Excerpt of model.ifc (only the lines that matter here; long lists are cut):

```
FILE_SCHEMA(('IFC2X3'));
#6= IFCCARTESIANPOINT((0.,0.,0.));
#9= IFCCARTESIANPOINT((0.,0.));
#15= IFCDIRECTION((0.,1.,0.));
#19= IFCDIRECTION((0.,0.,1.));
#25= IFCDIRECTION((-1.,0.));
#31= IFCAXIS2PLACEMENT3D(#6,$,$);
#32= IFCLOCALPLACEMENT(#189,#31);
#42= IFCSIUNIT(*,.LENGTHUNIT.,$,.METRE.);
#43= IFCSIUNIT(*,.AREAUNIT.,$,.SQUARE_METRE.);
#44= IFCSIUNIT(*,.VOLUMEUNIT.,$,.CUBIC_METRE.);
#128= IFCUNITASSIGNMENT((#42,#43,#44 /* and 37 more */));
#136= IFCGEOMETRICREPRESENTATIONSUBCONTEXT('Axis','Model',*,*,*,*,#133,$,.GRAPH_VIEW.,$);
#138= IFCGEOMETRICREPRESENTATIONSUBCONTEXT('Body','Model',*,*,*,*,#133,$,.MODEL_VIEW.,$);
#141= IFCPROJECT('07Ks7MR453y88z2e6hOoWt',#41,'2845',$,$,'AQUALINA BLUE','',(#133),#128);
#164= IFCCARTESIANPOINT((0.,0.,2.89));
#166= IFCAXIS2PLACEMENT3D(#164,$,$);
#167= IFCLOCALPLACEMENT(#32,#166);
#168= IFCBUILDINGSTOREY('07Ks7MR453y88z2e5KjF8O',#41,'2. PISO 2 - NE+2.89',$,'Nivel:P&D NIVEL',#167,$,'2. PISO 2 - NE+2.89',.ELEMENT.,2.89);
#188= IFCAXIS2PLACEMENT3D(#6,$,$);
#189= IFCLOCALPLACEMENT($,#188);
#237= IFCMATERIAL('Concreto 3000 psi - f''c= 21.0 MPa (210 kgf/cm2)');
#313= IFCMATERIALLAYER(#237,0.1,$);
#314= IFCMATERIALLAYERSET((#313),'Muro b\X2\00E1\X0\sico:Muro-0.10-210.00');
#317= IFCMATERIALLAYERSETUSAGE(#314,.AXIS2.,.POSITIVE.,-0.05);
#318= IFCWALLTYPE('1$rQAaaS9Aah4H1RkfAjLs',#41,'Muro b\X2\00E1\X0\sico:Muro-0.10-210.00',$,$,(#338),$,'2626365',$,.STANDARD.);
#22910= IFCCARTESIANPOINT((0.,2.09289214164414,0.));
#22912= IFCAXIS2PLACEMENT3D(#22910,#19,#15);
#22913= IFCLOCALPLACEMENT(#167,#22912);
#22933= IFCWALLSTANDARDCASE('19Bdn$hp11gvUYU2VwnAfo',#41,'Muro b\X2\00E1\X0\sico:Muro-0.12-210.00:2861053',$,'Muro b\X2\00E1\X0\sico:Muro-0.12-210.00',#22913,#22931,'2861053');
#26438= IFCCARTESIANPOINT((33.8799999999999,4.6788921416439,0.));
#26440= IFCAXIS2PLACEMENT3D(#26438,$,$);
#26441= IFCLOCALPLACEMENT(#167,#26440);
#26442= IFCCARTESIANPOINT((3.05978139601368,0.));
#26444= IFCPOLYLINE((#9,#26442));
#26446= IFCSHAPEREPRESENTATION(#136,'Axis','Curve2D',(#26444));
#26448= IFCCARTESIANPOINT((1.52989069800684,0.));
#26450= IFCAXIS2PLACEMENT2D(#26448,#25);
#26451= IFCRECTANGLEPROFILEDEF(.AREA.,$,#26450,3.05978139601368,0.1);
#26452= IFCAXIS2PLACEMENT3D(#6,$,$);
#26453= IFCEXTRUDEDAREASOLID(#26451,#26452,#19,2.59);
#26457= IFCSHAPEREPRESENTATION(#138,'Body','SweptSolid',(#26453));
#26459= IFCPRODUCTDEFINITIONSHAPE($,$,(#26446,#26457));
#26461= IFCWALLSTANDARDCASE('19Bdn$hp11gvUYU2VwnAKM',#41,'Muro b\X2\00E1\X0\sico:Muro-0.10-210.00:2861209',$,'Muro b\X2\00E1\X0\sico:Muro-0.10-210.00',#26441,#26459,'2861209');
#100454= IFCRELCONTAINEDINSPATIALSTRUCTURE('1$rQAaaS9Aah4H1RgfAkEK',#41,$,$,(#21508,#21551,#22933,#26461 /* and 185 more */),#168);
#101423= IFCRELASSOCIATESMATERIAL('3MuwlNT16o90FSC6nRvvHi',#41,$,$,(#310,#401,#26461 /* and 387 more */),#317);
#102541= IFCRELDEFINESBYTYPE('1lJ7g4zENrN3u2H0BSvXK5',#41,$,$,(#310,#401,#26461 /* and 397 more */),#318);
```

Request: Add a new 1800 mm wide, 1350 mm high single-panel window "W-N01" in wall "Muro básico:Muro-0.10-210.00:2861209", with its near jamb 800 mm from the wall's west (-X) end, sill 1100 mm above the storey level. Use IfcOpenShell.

```python
import numpy as np
import ifcopenshell
import ifcopenshell.api.feature
import ifcopenshell.api.geometry
import ifcopenshell.api.root
import ifcopenshell.api.spatial
import ifcopenshell.api.type
import ifcopenshell.geom
import ifcopenshell.util.element
import ifcopenshell.util.placement
import ifcopenshell.util.representation
import ifcopenshell.util.shape
import ifcopenshell.util.unit

model = ifcopenshell.open("model.ifc")
unit_scale = ifcopenshell.util.unit.calculate_unit_scale(model)
settings = ifcopenshell.geom.settings()


def volume(element):
    """Net volume in cubic metres, openings subtracted."""
    shape = ifcopenshell.geom.create_shape(settings, element)
    return ifcopenshell.util.shape.get_volume(shape.geometry)


wall = model.by_guid("19Bdn$hp11gvUYU2VwnAKM")
storey = ifcopenshell.util.element.get_container(wall, ifc_class="IfcBuildingStorey")
context = ifcopenshell.util.representation.get_context(model, "Model", "Body", "MODEL_VIEW")
before = volume(wall)

width, height, from_end, sill = 1.8, 1.35, 0.8, 1.1  # metres

# The wall runs along its own X axis, and the end named is its -X end.
wall_shape = ifcopenshell.geom.create_shape(settings, wall)
x, y, z = ifcopenshell.util.shape.get_vertices(wall_shape.geometry).T
start = x.min() + from_end
face, thickness = float(y.min()), float(y.max() - y.min())
wall_matrix = ifcopenshell.util.placement.get_local_placement(wall.ObjectPlacement)
level = ifcopenshell.util.placement.get_local_placement(storey.ObjectPlacement)[2, 3]


def in_wall(x, y):
    """Placement at x, y metres in the wall's axes, at sill height."""
    matrix = wall_matrix.copy()
    matrix[:, 3] = wall_matrix @ np.array([x / unit_scale, y / unit_scale, 0.0, 1.0])
    matrix[2, 3] = level + sill / unit_scale
    return matrix


# Opening: a box that overshoots both wall faces by 50 mm.
opening = ifcopenshell.api.root.create_entity(model, ifc_class="IfcOpeningElement")
box = ifcopenshell.api.geometry.add_wall_representation(
    model, context=context, length=width, height=height, thickness=thickness + 0.1
)
ifcopenshell.api.geometry.assign_representation(model, product=opening, representation=box)
ifcopenshell.api.geometry.edit_object_placement(model, product=opening, matrix=in_wall(start, face - 0.05), is_si=False)
ifcopenshell.api.feature.add_feature(model, feature=opening, element=wall)

window = ifcopenshell.api.root.create_entity(model, ifc_class="IfcWindow", name="W-N01")
window.OverallWidth, window.OverallHeight = width / unit_scale, height / unit_scale
body = ifcopenshell.api.geometry.add_window_representation(
    model,
    context=context,
    overall_width=window.OverallWidth,
    overall_height=window.OverallHeight,
    partition_type="SINGLE_PANEL",
)
ifcopenshell.api.geometry.assign_representation(model, product=window, representation=body)
ifcopenshell.api.spatial.assign_container(model, products=[window], relating_structure=storey)
fills = ifcopenshell.api.feature.add_filling(model, opening=opening, element=window)
fills.OwnerHistory = window.OwnerHistory  # required in IFC2X3

# IFC2X3 keeps the operation on the window style.
style = ifcopenshell.api.root.create_entity(model, ifc_class="IfcWindowStyle", name="W-N01")
style.OperationType, style.ConstructionType = "SINGLE_PANEL", "NOTDEFINED"
style.ParameterTakesPrecedence = style.Sizeable = False
ifcopenshell.api.type.assign_type(model, related_objects=[window], relating_type=style)

# Centre the window in the wall's thickness.
ifcopenshell.api.geometry.edit_object_placement(model, product=window, matrix=in_wall(start, face), is_si=False)
window_shape = ifcopenshell.geom.create_shape(settings, window)
depth = ifcopenshell.util.shape.get_vertices(window_shape.geometry)[:, 1]
offset = face + thickness / 2 - (depth.min() + depth.max()) / 2
ifcopenshell.api.geometry.edit_object_placement(model, product=window, matrix=in_wall(start, offset), is_si=False)

after = volume(wall)

print(f"wall volume {before:.3f} -> {after:.3f} m3")

model.write("model-out.ifc")
```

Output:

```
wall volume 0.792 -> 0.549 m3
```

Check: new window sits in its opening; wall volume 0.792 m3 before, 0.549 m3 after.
